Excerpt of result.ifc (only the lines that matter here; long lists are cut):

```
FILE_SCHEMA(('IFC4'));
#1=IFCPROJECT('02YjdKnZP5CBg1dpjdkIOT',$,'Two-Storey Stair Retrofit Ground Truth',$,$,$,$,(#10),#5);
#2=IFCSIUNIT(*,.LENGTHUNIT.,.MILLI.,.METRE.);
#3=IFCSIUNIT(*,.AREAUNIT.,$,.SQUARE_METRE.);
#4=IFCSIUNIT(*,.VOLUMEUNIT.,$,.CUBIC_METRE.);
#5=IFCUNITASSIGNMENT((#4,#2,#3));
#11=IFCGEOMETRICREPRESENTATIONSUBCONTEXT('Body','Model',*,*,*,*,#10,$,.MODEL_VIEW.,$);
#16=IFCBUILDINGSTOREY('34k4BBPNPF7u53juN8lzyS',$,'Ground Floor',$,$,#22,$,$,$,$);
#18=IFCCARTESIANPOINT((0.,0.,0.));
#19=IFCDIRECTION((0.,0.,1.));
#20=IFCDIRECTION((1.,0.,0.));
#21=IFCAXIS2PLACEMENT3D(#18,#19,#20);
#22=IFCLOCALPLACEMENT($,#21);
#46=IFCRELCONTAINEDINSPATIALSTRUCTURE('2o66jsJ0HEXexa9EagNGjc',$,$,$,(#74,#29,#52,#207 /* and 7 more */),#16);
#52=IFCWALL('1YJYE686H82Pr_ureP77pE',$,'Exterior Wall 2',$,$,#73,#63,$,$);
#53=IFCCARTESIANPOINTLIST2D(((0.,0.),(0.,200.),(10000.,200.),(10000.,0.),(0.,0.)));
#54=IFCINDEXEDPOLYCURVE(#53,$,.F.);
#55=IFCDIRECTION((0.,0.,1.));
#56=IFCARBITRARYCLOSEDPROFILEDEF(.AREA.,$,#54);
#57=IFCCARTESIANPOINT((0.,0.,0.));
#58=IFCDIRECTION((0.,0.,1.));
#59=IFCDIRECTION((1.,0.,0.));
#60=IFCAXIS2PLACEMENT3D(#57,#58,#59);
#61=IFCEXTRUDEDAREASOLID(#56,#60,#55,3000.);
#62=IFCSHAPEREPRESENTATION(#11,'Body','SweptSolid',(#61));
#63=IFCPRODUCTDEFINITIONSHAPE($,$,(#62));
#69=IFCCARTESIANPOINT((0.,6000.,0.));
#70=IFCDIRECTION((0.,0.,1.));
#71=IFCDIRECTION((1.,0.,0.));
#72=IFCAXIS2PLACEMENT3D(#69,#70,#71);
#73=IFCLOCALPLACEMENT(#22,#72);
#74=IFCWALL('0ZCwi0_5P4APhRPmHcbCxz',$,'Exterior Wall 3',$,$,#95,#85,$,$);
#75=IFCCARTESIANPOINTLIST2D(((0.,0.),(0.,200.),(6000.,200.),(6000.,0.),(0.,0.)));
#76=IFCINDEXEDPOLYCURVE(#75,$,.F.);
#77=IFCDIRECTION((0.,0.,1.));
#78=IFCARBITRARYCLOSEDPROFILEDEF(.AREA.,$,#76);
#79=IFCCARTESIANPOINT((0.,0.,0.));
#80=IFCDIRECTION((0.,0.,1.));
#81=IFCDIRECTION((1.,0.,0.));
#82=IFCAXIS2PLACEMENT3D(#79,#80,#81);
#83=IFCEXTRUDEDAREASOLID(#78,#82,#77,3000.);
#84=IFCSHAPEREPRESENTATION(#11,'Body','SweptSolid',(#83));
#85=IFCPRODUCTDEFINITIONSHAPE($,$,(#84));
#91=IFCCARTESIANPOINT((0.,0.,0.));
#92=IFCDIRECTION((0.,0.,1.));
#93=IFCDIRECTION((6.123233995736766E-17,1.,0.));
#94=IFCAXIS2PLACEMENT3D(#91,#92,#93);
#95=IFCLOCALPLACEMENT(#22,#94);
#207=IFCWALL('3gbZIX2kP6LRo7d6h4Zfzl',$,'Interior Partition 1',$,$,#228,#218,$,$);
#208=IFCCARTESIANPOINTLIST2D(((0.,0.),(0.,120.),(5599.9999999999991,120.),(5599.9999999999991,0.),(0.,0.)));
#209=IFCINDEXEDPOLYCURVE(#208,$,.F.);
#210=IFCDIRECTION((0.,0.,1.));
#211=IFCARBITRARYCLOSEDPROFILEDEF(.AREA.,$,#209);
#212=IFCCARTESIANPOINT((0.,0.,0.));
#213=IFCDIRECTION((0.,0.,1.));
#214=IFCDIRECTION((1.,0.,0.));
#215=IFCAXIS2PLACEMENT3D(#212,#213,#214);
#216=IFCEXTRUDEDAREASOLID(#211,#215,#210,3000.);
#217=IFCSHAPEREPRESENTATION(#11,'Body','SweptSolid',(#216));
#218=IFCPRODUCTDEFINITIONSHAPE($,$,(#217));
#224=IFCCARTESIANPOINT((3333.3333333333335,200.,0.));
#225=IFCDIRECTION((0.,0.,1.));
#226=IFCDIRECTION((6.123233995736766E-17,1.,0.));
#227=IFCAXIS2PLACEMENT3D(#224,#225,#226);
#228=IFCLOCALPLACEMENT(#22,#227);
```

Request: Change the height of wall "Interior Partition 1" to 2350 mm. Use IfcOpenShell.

```python
import ifcopenshell
import ifcopenshell.geom
import ifcopenshell.util.representation
import ifcopenshell.util.shape
import ifcopenshell.util.unit

model = ifcopenshell.open("result.ifc")
unit_scale = ifcopenshell.util.unit.calculate_unit_scale(model)
settings = ifcopenshell.geom.settings()


def volume(element):
    """Net volume in cubic metres, openings subtracted."""
    shape = ifcopenshell.geom.create_shape(settings, element)
    return ifcopenshell.util.shape.get_volume(shape.geometry)


wall = model.by_guid("3gbZIX2kP6LRo7d6h4Zfzl")
before = volume(wall)

body = ifcopenshell.util.representation.get_representation(wall, "Model", "Body")
solid = body.Items[0]
old_height = solid.Depth
solid.Depth = 2.35 / unit_scale
after = volume(wall)

print(f"height {old_height:g} -> {solid.Depth:g}, volume {before:.3f} -> {after:.3f} m3")

model.write("result-out.ifc")
```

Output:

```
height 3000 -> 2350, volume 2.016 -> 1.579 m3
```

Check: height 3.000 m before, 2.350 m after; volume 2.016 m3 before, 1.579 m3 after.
